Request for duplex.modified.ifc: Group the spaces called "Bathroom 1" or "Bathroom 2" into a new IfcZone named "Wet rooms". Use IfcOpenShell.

First a look at what the model holds.

```python
import ifcopenshell

model = ifcopenshell.open("duplex.modified.ifc")
print(model.schema)
seen = {}
for space in model.by_type("IfcSpace"):
    seen[space.LongName] = seen.get(space.LongName, 0) + 1
for name, count in sorted(seen.items(), key=str):
    print(count, "x", name)
print("zones:", [z.Name for z in model.by_type("IfcZone")][:20])
```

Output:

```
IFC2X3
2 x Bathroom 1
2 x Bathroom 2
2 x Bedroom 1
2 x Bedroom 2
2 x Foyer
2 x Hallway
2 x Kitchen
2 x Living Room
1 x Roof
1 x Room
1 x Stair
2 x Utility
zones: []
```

```python
import ifcopenshell
import ifcopenshell.api.group
import ifcopenshell.api.root

model = ifcopenshell.open("duplex.modified.ifc")

names = {"Bathroom 1", "Bathroom 2"}
spaces = [s for s in model.by_type("IfcSpace") if s.LongName in names]

zone = ifcopenshell.api.root.create_entity(model, ifc_class="IfcZone", name="Wet rooms")
ifcopenshell.api.group.assign_group(model, products=spaces, group=zone)
print(len(spaces), "spaces in", zone.Name)

model.write("duplex.modified-out.ifc")
```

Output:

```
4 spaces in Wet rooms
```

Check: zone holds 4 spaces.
